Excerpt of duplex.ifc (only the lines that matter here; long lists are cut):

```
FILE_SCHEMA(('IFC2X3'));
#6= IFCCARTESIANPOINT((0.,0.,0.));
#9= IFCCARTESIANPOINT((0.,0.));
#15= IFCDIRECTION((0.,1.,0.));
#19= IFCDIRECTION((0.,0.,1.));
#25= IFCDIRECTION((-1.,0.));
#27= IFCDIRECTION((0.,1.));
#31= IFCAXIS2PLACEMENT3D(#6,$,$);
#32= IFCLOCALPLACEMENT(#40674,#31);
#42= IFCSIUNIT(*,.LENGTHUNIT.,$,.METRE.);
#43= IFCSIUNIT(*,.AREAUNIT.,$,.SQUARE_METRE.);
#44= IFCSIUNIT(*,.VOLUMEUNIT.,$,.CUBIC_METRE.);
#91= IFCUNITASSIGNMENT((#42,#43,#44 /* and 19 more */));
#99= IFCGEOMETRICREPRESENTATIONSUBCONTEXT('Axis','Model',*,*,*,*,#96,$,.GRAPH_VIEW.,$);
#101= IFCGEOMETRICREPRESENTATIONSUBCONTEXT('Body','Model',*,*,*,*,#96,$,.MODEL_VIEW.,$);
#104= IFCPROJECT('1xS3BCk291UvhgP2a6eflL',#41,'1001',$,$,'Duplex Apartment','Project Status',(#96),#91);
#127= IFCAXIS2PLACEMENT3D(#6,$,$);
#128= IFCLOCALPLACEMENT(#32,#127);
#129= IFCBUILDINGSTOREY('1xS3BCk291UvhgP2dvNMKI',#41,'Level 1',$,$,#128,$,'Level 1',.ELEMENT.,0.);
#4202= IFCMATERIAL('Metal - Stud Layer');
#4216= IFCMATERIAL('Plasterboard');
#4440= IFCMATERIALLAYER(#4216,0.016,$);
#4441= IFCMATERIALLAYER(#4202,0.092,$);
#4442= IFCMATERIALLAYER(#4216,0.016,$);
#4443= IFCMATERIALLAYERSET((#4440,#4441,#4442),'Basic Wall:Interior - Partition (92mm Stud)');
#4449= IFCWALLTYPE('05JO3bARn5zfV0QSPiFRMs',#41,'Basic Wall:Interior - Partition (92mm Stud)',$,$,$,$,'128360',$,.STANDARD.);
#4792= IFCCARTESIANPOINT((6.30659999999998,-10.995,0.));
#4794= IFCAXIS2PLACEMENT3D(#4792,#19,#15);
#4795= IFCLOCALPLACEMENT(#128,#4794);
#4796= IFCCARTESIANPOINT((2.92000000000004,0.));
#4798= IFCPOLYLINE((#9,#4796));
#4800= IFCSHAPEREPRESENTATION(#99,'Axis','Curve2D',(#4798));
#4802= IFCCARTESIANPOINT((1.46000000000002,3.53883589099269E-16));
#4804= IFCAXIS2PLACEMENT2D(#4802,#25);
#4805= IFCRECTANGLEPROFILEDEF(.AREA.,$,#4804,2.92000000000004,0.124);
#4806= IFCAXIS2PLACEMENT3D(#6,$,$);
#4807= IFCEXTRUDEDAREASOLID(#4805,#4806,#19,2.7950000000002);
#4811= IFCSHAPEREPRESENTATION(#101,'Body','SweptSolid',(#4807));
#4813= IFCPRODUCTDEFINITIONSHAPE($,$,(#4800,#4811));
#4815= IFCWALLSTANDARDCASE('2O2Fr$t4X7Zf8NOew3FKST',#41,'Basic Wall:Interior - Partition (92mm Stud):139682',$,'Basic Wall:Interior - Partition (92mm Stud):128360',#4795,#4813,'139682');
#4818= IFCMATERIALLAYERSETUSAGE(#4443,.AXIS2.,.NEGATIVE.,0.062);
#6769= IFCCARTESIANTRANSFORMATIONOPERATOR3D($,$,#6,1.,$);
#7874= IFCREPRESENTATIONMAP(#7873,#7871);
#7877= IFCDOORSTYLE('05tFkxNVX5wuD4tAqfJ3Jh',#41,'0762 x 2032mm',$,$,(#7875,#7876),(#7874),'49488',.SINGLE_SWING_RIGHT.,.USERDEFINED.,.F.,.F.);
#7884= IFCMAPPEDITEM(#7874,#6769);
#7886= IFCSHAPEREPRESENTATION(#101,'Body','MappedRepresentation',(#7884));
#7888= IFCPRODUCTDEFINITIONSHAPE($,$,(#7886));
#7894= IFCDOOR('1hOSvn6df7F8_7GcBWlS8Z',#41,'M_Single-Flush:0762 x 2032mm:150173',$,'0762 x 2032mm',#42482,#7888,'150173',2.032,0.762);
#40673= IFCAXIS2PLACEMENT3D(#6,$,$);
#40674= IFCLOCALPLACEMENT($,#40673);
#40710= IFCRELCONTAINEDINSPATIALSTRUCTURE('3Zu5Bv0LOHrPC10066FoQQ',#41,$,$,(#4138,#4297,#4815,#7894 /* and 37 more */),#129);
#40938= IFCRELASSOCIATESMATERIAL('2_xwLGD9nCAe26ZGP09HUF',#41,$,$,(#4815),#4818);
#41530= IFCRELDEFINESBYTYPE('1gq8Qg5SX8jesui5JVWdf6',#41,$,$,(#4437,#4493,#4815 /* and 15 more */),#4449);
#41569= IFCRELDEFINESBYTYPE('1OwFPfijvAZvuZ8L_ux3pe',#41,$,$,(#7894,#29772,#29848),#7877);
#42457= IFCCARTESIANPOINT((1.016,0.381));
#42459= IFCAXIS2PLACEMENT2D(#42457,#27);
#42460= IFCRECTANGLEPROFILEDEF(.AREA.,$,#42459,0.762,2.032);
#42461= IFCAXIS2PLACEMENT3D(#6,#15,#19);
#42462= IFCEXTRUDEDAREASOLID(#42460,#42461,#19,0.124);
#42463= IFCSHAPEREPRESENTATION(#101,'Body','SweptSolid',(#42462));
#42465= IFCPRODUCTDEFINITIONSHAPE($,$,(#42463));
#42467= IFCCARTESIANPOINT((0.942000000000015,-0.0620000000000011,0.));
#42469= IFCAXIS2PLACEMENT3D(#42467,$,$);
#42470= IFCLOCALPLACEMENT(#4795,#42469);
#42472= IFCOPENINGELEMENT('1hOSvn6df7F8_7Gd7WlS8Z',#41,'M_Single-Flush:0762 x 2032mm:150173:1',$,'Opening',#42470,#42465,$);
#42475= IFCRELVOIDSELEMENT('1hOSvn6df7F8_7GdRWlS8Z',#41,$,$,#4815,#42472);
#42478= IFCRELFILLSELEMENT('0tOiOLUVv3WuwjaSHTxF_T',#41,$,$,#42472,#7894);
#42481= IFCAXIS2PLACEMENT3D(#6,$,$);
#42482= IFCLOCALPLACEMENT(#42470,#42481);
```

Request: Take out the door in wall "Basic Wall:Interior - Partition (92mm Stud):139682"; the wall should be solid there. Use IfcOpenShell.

```python
import ifcopenshell
import ifcopenshell.api.feature
import ifcopenshell.api.root
import ifcopenshell.geom
import ifcopenshell.util.shape

model = ifcopenshell.open("duplex.ifc")
settings = ifcopenshell.geom.settings()


def volume(element):
    """Net volume in cubic metres, openings subtracted."""
    shape = ifcopenshell.geom.create_shape(settings, element)
    return ifcopenshell.util.shape.get_volume(shape.geometry)


door = model.by_guid("1hOSvn6df7F8_7GcBWlS8Z")
opening = door.FillsVoids[0].RelatingOpeningElement
wall = opening.VoidsElements[0].RelatingBuildingElement
before = volume(wall)

ifcopenshell.api.root.remove_product(model, product=door)
ifcopenshell.api.feature.remove_feature(model, feature=opening)

after = volume(wall)

print(f"wall volume {before:.3f} -> {after:.3f} m3")

model.write("duplex-out.ifc")
```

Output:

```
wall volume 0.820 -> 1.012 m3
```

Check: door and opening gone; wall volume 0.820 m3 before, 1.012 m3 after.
